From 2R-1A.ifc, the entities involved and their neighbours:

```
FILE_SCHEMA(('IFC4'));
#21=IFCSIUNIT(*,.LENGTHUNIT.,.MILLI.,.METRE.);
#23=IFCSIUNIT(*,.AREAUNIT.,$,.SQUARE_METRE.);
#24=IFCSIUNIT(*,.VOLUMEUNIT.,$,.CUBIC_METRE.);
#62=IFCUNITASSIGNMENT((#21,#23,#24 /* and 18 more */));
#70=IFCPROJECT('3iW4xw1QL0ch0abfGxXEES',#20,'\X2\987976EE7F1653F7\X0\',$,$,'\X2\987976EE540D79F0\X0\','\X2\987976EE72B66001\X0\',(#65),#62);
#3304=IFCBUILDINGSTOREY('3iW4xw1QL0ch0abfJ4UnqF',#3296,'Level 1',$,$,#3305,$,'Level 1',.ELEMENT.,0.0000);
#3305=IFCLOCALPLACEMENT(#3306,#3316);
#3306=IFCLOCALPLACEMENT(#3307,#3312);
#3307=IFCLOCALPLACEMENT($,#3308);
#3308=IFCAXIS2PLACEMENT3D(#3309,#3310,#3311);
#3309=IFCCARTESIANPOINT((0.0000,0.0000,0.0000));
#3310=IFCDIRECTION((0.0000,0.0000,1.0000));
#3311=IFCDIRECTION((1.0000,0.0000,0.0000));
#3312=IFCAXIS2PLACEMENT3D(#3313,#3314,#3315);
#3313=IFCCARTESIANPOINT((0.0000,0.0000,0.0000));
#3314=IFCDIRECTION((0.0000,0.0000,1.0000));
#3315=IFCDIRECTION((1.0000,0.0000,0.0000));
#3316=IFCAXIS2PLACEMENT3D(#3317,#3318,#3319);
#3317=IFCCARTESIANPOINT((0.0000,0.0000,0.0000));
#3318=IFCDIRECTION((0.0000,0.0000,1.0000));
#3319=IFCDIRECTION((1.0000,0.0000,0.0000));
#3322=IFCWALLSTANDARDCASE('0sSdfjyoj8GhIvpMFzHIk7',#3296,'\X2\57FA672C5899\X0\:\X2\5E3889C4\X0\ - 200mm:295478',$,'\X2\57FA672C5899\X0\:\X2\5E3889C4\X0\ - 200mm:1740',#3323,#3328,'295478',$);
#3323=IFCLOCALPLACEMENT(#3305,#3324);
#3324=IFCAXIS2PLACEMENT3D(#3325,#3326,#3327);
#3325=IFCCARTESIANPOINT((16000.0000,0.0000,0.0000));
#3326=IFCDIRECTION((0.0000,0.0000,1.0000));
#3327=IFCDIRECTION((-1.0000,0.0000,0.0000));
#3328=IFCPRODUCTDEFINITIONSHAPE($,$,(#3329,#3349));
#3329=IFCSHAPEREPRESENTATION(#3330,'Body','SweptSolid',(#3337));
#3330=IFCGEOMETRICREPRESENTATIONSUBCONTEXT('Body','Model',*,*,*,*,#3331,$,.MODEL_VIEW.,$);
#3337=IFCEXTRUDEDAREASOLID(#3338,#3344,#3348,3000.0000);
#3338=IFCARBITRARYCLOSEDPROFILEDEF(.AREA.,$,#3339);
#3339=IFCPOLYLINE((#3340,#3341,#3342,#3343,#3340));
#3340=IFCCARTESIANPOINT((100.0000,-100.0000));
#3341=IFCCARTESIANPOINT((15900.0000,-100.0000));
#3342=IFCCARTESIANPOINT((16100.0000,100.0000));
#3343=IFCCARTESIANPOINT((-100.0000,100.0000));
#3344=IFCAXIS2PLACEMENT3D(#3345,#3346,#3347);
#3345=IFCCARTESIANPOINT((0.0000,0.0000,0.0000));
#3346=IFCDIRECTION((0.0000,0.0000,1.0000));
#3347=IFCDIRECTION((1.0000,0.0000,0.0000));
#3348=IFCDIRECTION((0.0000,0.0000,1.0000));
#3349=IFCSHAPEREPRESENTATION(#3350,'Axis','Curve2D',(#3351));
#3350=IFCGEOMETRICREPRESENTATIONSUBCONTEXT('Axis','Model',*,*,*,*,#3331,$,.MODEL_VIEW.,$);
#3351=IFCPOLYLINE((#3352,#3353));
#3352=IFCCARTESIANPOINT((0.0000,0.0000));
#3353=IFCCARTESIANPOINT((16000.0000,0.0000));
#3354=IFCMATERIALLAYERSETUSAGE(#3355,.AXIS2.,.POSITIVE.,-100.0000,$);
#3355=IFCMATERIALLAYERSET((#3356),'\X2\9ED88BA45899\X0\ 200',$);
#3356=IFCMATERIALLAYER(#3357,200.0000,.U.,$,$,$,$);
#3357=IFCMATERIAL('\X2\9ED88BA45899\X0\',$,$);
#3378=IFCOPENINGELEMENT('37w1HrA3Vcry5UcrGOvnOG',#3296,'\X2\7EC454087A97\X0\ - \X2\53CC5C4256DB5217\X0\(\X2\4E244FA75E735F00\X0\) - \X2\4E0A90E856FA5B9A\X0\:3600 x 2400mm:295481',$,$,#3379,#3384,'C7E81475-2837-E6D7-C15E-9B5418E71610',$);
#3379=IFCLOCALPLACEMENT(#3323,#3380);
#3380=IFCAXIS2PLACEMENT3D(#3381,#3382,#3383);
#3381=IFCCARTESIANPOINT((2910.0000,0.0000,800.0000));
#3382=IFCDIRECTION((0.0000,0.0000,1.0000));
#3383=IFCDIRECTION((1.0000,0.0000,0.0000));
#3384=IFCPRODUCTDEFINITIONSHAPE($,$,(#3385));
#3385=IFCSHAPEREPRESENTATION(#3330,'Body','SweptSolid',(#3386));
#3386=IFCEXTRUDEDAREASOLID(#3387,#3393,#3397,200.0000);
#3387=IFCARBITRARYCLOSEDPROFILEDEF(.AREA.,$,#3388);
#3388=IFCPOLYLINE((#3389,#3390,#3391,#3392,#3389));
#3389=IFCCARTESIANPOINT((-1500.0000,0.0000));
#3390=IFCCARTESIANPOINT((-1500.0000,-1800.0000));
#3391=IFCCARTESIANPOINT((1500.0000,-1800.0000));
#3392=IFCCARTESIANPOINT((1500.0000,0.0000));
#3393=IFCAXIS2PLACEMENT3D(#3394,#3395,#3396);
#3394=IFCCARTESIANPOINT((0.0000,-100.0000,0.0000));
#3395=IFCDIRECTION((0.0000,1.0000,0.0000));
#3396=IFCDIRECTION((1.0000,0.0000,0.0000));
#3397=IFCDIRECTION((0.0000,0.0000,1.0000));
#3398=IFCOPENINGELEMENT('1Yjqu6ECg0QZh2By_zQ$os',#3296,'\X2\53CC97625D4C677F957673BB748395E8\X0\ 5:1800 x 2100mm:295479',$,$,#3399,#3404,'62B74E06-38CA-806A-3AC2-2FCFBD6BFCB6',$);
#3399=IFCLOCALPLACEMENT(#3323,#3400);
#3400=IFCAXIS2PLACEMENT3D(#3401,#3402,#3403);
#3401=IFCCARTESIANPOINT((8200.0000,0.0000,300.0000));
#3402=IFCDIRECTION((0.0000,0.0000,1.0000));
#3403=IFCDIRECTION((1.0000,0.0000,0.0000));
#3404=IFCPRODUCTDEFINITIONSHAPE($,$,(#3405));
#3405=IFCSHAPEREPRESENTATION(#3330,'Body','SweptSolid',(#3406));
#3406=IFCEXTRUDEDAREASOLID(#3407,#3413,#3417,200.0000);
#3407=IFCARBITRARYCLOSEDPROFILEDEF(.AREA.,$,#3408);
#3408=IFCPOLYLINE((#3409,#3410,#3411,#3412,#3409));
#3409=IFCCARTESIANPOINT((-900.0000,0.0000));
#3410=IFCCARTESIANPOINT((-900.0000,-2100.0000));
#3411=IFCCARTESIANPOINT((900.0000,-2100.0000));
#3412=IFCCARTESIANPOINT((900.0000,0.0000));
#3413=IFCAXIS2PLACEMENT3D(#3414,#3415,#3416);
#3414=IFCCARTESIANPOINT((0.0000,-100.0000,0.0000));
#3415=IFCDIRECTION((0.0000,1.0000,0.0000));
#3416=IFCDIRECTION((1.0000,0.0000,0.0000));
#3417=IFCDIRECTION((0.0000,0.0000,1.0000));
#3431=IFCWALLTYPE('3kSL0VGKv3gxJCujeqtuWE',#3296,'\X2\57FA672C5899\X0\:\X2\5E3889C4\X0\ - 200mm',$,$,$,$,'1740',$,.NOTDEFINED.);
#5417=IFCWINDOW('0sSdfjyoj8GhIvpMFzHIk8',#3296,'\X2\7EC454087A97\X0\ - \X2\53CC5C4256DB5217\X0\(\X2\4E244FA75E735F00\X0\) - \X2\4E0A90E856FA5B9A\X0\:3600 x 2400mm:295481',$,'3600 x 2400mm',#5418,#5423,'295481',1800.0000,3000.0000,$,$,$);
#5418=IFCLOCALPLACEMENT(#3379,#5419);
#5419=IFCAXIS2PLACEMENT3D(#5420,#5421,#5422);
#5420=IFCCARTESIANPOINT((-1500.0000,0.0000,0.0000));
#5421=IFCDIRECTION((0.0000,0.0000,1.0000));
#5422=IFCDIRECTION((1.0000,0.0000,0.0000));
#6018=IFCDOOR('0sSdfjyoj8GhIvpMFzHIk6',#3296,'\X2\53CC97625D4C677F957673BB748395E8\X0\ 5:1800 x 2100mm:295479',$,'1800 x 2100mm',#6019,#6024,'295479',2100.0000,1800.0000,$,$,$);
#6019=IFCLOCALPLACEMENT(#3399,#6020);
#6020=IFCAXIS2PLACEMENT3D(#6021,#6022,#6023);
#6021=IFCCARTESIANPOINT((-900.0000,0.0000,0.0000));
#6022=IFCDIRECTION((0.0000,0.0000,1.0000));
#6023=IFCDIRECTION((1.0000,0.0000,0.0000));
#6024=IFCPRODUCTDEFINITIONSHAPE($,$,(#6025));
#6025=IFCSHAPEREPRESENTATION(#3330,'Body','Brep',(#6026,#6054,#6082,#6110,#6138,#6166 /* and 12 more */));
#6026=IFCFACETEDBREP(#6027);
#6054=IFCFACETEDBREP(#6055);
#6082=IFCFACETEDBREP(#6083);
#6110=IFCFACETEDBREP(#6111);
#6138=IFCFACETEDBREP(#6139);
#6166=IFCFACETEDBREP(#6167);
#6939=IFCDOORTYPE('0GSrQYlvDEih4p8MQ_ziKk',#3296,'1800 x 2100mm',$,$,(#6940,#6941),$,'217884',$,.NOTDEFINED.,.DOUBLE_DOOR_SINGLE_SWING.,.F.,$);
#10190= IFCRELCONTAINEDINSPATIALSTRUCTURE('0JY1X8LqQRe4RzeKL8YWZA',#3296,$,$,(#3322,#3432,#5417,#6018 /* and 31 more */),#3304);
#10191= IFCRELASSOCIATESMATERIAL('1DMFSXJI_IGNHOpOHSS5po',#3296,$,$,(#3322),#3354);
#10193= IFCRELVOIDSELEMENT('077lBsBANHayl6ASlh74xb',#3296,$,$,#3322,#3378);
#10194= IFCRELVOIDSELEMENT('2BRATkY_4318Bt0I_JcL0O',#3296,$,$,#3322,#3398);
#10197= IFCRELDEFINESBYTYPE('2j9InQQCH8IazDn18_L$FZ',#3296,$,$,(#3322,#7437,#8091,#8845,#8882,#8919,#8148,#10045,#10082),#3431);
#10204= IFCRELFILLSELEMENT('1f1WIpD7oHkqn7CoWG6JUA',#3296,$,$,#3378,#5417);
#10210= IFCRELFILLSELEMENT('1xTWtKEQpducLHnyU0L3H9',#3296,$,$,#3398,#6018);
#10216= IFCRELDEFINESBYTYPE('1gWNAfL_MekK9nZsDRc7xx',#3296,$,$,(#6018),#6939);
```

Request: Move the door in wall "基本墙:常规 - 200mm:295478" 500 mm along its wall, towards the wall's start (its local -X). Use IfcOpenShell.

```python
import ifcopenshell
import ifcopenshell.api.geometry
import ifcopenshell.util.placement
import ifcopenshell.util.unit

model = ifcopenshell.open("2R-1A.ifc")
unit_scale = ifcopenshell.util.unit.calculate_unit_scale(model)

door = model.by_guid("0sSdfjyoj8GhIvpMFzHIk6")
opening = door.FillsVoids[0].RelatingOpeningElement
wall = opening.VoidsElements[0].RelatingBuildingElement

wall_matrix = ifcopenshell.util.placement.get_local_placement(wall.ObjectPlacement)
shift = wall_matrix[:3, 0] * -0.5 / unit_scale
before = ifcopenshell.util.placement.get_local_placement(door.ObjectPlacement)[:3, 3].copy()

# The door is placed relative to its opening, so it follows when the opening moves.
matrix = ifcopenshell.util.placement.get_local_placement(opening.ObjectPlacement)
matrix[:3, 3] += shift
ifcopenshell.api.geometry.edit_object_placement(
    model, product=opening, matrix=matrix, is_si=False, should_transform_children=True
)

after = ifcopenshell.util.placement.get_local_placement(door.ObjectPlacement)[:3, 3]
print("door moved by", (after - before).round(3) + 0.0)

model.write("2R-1A_rev.ifc")
```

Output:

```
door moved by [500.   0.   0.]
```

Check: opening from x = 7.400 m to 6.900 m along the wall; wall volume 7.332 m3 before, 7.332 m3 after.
